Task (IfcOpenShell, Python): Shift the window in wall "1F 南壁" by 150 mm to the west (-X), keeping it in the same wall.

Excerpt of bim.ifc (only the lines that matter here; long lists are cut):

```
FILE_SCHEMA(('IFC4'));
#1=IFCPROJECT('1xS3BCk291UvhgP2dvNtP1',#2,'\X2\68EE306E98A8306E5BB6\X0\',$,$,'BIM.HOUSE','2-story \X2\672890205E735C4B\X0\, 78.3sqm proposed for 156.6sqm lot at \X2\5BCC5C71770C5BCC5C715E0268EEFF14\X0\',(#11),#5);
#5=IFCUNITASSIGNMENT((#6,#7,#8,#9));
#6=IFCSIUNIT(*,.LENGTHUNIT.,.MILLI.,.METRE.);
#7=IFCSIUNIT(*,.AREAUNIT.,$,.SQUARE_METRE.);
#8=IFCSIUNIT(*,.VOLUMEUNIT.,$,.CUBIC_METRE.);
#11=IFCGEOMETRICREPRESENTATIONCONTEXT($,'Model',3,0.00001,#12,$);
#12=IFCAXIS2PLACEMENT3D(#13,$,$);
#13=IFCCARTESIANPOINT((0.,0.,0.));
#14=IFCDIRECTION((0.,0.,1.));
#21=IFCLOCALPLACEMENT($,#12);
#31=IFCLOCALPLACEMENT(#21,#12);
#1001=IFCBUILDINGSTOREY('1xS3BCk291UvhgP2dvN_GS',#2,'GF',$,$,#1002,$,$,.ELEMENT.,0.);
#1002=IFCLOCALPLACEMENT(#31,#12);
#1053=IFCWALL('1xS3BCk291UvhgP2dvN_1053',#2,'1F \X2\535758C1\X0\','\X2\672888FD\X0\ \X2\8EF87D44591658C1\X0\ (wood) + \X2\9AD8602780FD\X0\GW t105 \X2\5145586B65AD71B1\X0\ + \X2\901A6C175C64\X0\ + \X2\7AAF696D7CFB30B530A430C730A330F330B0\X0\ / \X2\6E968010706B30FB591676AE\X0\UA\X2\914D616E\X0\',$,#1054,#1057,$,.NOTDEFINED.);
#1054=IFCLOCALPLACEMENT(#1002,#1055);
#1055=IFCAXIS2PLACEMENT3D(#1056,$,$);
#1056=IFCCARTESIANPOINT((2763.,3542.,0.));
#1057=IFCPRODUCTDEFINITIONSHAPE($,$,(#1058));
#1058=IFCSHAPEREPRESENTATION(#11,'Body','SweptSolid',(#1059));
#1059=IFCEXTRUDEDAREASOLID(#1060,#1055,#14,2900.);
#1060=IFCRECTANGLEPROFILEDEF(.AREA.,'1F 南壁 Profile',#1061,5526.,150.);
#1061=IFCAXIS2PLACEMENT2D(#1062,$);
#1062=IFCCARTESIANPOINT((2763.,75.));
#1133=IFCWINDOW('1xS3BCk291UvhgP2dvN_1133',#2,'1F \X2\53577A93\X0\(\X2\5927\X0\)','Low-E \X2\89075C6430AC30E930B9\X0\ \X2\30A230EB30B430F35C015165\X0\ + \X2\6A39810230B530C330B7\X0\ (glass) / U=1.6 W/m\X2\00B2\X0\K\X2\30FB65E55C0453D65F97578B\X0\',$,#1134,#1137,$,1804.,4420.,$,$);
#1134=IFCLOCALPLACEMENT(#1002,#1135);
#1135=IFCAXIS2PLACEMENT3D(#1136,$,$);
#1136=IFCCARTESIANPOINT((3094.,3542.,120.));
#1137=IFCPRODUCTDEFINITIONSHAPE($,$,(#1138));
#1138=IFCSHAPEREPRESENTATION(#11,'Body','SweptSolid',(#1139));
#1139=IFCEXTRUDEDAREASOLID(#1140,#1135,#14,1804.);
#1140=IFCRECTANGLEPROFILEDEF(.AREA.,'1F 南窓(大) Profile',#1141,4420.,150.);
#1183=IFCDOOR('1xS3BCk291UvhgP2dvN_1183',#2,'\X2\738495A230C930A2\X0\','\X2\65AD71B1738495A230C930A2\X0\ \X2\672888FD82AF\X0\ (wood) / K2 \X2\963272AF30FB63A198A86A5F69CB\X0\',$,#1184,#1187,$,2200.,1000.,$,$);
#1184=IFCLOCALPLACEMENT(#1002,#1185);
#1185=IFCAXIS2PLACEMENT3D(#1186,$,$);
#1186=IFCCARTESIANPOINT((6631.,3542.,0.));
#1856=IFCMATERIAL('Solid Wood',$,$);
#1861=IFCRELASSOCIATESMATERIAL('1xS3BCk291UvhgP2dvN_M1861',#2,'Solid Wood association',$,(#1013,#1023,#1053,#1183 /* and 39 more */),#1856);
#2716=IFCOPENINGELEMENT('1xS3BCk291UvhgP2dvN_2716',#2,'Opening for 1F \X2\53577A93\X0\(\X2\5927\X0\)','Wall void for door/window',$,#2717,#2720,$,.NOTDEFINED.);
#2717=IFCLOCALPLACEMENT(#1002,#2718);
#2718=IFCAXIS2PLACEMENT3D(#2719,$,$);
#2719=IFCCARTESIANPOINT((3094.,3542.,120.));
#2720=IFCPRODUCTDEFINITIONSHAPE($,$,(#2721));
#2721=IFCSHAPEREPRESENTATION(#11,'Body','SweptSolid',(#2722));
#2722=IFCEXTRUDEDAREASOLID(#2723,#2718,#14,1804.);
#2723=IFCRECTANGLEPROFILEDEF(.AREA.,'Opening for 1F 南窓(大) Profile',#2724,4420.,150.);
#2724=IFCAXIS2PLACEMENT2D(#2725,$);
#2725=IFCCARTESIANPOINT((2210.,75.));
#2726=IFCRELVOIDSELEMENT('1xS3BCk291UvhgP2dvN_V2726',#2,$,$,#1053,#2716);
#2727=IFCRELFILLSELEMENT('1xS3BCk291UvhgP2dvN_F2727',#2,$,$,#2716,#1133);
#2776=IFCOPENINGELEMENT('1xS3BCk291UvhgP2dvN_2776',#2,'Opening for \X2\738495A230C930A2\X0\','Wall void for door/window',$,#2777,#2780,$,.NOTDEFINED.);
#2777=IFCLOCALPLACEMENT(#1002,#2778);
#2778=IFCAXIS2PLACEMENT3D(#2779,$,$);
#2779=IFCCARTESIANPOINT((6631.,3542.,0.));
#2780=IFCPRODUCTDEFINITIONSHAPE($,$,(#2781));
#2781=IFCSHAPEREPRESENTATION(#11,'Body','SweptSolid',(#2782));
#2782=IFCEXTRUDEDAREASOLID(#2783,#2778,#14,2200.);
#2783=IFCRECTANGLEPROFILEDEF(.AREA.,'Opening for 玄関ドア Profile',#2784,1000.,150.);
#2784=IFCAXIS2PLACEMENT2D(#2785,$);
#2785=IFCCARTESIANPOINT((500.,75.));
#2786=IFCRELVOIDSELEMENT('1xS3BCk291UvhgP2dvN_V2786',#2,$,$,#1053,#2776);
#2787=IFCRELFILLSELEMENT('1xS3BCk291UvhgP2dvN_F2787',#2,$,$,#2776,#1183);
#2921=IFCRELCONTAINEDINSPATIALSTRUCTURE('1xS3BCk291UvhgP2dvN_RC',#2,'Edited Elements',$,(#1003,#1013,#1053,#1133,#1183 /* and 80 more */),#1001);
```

```python
import ifcopenshell
import ifcopenshell.api.geometry
import ifcopenshell.util.placement

model = ifcopenshell.open("bim.ifc")

window = model.by_guid("1xS3BCk291UvhgP2dvN_1133")
opening = window.FillsVoids[0].RelatingOpeningElement
wall = opening.VoidsElements[0].RelatingBuildingElement

wall_matrix = ifcopenshell.util.placement.get_local_placement(wall.ObjectPlacement)
shift = wall_matrix[:3, 0] * -150.0
before = ifcopenshell.util.placement.get_local_placement(window.ObjectPlacement)[:3, 3].copy()

# The window is not placed relative to its opening, so move both.
for product in (opening, window):
    matrix = ifcopenshell.util.placement.get_local_placement(product.ObjectPlacement)
    matrix[:3, 3] += shift
    ifcopenshell.api.geometry.edit_object_placement(model, product=product, matrix=matrix, is_si=False)

after = ifcopenshell.util.placement.get_local_placement(window.ObjectPlacement)[:3, 3]
print("window moved by", (after - before).round(3) + 0.0)

model.write("bim_v2.ifc")
```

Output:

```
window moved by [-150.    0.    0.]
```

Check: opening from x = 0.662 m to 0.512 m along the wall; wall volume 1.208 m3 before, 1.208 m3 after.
